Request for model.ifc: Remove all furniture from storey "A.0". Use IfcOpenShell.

First a look at what the model holds.

```python
import ifcopenshell
import ifcopenshell.util.element

model = ifcopenshell.open("model.ifc")
print(model.schema)
storey = next(s for s in model.by_type("IfcBuildingStorey") if s.Name == "A.0")
furniture = [e for e in ifcopenshell.util.element.get_decomposition(storey) if e.is_a("IfcFurnishingElement")]
seen = {}
for e in furniture:
    element_type = ifcopenshell.util.element.get_type(e)
    name = element_type.Name if element_type not in (None, e) else None
    seen[name] = seen.get(name, 0) + 1
for name, count in sorted(seen.items(), key=str):
    print(count, "x", name)
```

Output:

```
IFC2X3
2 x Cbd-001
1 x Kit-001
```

```python
import ifcopenshell
import ifcopenshell.api.root
import ifcopenshell.util.element

model = ifcopenshell.open("model.ifc")

storey = next(s for s in model.by_type("IfcBuildingStorey") if s.Name == "A.0")
furniture = [e for e in ifcopenshell.util.element.get_decomposition(storey) if e.is_a("IfcFurnishingElement")]

for e in furniture:
    ifcopenshell.api.root.remove_product(model, product=e)
print(len(furniture), "removed")

model.write("model-out.ifc")
```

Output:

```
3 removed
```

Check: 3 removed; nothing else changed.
